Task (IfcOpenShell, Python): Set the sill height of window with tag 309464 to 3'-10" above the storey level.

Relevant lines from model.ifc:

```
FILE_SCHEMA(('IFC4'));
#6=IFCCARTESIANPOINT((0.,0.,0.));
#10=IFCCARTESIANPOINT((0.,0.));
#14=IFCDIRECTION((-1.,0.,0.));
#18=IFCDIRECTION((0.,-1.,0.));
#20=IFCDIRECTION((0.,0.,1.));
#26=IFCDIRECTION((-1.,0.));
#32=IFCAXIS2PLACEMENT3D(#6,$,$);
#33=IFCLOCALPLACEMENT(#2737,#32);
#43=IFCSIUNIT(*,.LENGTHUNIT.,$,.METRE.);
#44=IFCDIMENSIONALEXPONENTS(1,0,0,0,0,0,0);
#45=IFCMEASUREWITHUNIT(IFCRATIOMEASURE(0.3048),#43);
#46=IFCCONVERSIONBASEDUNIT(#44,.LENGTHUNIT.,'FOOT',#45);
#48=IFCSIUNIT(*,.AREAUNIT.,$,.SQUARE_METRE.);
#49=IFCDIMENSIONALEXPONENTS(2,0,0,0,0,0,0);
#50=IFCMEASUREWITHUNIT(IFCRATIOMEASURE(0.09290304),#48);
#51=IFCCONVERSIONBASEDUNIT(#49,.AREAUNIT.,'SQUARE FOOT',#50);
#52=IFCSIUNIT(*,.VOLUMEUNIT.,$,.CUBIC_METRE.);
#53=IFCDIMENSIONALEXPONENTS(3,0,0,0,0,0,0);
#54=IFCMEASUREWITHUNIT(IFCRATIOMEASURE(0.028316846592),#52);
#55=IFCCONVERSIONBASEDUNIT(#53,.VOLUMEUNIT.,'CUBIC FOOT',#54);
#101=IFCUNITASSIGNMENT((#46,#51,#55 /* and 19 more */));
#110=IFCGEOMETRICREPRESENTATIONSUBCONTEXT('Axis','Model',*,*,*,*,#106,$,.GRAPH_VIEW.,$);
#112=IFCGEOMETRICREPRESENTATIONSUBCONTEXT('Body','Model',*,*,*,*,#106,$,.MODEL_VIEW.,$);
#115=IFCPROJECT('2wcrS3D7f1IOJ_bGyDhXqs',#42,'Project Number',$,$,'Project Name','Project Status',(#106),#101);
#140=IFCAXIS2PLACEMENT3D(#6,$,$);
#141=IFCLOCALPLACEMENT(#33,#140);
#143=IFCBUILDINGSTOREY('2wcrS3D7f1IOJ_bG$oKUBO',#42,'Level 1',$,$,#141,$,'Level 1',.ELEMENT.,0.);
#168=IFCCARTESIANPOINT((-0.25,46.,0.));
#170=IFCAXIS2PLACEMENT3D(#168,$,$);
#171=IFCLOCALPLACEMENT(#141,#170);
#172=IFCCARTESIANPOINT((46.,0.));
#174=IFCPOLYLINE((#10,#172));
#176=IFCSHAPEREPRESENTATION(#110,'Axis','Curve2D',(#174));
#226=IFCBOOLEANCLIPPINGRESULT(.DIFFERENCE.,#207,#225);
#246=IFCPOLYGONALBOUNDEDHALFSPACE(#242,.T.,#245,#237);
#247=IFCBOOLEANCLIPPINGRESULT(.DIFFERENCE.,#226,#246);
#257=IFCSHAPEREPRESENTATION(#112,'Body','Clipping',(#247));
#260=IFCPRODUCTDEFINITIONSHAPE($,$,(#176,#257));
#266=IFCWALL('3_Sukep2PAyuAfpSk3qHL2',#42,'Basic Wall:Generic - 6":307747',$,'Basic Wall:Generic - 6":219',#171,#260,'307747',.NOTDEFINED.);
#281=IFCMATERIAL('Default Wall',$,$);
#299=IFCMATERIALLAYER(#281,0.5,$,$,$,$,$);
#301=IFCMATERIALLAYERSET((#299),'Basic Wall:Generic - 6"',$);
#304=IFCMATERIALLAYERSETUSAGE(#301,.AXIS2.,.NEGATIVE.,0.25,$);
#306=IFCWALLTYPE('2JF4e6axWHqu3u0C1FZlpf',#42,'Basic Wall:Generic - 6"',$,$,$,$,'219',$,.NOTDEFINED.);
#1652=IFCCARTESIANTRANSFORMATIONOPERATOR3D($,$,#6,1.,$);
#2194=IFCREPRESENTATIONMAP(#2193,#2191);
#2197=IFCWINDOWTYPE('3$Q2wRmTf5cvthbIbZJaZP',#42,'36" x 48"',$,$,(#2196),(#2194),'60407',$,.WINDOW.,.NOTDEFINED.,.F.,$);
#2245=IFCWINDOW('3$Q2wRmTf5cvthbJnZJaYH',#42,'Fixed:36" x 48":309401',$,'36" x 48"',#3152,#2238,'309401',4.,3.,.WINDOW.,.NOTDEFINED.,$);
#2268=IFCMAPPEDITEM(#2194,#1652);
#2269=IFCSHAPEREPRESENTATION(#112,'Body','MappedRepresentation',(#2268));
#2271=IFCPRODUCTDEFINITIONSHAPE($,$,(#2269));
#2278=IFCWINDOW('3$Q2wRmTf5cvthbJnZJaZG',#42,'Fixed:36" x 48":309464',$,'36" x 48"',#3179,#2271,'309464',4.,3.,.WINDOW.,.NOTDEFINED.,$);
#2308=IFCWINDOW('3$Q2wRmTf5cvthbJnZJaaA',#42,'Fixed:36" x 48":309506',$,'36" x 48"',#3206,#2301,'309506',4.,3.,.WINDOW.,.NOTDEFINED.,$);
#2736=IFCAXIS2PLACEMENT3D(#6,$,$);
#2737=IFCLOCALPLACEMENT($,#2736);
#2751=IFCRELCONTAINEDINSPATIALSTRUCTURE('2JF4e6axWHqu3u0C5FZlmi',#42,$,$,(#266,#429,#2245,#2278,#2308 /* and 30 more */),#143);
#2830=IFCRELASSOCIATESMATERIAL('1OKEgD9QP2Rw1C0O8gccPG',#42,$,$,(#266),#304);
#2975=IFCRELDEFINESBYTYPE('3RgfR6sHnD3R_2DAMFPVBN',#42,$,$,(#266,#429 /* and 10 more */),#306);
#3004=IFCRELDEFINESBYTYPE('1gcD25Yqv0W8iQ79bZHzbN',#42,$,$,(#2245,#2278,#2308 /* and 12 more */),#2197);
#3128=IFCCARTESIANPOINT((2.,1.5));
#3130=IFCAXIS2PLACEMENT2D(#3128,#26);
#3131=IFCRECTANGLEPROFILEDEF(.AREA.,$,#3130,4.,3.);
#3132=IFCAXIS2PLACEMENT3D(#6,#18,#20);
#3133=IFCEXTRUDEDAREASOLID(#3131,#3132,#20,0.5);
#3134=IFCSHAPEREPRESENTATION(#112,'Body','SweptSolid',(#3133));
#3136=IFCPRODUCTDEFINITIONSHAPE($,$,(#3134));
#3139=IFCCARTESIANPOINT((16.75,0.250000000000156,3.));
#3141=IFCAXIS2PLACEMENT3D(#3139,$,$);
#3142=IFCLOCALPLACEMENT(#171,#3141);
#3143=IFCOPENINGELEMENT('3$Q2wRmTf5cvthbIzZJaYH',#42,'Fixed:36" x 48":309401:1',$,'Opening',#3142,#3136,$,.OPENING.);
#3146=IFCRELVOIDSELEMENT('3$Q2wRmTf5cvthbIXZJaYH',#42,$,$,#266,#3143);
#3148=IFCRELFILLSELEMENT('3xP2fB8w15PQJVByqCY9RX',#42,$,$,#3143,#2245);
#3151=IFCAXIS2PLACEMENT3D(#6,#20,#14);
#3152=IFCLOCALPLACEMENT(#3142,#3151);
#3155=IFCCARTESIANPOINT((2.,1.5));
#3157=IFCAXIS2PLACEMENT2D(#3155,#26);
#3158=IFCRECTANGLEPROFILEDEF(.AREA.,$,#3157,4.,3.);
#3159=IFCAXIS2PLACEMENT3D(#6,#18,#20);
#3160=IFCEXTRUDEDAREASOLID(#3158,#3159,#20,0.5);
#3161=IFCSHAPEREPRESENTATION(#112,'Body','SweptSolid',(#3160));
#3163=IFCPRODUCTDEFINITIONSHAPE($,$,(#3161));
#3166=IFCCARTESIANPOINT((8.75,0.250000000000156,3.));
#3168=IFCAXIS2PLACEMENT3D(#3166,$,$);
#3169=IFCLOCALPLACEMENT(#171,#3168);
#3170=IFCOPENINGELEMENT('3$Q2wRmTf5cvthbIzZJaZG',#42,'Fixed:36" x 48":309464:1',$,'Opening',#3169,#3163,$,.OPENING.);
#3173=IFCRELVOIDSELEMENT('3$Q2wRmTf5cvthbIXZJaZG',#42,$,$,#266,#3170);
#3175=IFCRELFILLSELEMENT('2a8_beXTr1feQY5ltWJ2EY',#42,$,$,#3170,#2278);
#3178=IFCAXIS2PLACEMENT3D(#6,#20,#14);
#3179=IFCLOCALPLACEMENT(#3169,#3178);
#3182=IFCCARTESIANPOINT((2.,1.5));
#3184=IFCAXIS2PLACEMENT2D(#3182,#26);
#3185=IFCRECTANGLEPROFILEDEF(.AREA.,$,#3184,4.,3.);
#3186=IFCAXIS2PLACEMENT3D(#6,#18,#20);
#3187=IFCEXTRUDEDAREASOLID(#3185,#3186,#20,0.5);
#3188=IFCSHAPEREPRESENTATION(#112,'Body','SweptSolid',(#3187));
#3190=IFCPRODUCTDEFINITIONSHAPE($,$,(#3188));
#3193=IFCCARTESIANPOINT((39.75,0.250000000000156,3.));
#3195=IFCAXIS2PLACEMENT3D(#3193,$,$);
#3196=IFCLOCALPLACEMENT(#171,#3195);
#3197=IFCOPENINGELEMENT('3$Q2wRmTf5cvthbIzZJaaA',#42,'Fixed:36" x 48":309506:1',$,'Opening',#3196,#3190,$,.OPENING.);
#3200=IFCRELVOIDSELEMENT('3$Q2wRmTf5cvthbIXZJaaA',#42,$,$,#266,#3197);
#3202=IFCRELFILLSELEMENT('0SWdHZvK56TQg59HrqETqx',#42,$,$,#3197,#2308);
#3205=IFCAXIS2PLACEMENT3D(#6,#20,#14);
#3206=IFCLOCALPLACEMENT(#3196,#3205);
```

```python
import numpy as np
import ifcopenshell
import ifcopenshell.api.geometry
import ifcopenshell.geom
import ifcopenshell.util.element
import ifcopenshell.util.placement
import ifcopenshell.util.shape
import ifcopenshell.util.unit

model = ifcopenshell.open("model.ifc")
unit_scale = ifcopenshell.util.unit.calculate_unit_scale(model)

window = model.by_guid("3$Q2wRmTf5cvthbJnZJaZG")
opening = window.FillsVoids[0].RelatingOpeningElement
storey = ifcopenshell.util.element.get_container(window, ifc_class="IfcBuildingStorey")
level = ifcopenshell.util.placement.get_local_placement(storey.ObjectPlacement)[2, 3]

# The opening's origin need not be at the sill, so measure its lowest point.
shape = ifcopenshell.geom.create_shape(ifcopenshell.geom.settings(), opening)
bottom = ifcopenshell.util.shape.get_shape_bottom_elevation(shape, shape.geometry) / unit_scale
dz = level + 46 * 0.0254 / unit_scale - bottom

shift = np.array([0.0, 0.0, dz])
# The window is placed relative to its opening, so it follows when the opening moves.
matrix = ifcopenshell.util.placement.get_local_placement(opening.ObjectPlacement)
matrix[:3, 3] += shift
ifcopenshell.api.geometry.edit_object_placement(
    model, product=opening, matrix=matrix, is_si=False, should_transform_children=True
)

print(f"moved by {dz * unit_scale:+.3f} m")

model.write("model_updated.ifc")
```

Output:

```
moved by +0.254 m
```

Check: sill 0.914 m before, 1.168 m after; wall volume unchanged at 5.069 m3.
